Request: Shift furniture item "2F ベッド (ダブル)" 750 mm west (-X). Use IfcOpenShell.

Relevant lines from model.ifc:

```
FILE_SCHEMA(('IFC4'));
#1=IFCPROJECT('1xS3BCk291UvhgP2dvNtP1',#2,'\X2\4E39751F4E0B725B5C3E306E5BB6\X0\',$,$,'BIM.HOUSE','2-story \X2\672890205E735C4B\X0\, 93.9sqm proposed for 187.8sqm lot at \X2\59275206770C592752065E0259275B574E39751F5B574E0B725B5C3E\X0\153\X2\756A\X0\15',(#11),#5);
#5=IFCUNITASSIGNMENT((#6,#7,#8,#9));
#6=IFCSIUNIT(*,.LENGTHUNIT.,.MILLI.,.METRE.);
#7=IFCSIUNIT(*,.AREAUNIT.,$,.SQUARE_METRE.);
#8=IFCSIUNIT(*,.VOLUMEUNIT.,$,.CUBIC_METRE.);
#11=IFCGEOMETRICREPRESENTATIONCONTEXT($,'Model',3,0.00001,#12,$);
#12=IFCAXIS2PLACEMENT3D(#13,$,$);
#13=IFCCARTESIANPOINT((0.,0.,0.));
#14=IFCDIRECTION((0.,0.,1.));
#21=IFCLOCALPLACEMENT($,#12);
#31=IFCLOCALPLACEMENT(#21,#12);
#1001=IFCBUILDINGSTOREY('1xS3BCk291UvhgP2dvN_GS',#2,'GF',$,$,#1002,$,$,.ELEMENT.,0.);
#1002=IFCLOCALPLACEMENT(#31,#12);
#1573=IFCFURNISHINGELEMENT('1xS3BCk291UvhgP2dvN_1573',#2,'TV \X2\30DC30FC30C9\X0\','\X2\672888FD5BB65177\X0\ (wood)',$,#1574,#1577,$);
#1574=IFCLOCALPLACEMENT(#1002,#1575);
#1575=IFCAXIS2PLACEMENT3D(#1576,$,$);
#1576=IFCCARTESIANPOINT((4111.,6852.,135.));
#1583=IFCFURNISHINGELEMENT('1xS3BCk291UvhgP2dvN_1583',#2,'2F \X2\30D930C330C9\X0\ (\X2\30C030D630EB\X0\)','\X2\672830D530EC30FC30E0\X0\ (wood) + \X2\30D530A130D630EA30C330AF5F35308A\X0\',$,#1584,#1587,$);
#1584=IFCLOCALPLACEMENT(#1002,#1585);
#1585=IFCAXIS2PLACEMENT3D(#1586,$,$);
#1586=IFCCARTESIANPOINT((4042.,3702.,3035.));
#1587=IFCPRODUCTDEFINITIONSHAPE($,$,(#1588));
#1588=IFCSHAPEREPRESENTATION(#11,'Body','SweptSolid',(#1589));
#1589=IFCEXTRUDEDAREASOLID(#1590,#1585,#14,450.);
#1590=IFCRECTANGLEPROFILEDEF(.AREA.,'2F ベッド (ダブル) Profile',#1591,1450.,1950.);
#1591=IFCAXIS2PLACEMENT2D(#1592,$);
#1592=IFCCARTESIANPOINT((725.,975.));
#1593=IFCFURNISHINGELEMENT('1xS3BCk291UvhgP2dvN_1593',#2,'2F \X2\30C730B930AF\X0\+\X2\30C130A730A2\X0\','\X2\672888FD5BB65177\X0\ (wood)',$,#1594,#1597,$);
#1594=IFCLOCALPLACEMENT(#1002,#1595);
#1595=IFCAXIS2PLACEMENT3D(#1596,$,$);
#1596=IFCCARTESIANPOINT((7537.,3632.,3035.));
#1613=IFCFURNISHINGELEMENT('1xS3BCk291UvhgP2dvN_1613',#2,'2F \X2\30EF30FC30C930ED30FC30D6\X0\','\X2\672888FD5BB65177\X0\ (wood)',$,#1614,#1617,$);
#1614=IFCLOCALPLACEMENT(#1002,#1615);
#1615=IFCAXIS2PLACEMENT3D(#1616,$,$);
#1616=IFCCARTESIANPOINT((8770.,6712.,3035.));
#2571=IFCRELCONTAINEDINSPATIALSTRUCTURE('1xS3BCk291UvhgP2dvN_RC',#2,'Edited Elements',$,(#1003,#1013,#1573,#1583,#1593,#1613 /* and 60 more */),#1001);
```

```python
import ifcopenshell
import ifcopenshell.api.geometry
import ifcopenshell.util.placement
import ifcopenshell.util.unit

model = ifcopenshell.open("model.ifc")
unit_scale = ifcopenshell.util.unit.calculate_unit_scale(model)

item = model.by_guid("1xS3BCk291UvhgP2dvN_1583")
matrix = ifcopenshell.util.placement.get_local_placement(item.ObjectPlacement)
matrix[0, 3] -= 0.75 / unit_scale
ifcopenshell.api.geometry.edit_object_placement(model, product=item, matrix=matrix, is_si=False)

print(ifcopenshell.util.placement.get_local_placement(item.ObjectPlacement).round(3) + 0.0)

model.write("model_edited.ifc")
```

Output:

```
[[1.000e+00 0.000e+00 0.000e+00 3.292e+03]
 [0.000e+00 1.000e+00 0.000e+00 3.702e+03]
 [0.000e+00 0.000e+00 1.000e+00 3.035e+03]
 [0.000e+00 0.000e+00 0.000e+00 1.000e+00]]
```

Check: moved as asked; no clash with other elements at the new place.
